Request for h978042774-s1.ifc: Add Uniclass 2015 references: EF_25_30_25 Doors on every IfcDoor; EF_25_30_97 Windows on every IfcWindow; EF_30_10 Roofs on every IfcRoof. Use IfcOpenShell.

First a look at what the model holds.

```python
import ifcopenshell

model = ifcopenshell.open("h978042774-s1.ifc")
print(model.schema)
print("classifications:", [c.Name for c in model.by_type("IfcClassification")])
for ifc_class in ("IfcDoor", "IfcRoof", "IfcStair", "IfcWall", "IfcWindow"):
    print(ifc_class, len(model.by_type(ifc_class)))
```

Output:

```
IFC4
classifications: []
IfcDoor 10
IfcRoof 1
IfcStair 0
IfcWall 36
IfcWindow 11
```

```python
import ifcopenshell
import ifcopenshell.api.classification

model = ifcopenshell.open("h978042774-s1.ifc")

system = ifcopenshell.api.classification.add_classification(model, classification="Uniclass 2015")

codes = {
    "IfcDoor": ("EF_25_30_25", "Doors"),
    "IfcWindow": ("EF_25_30_97", "Windows"),
    "IfcRoof": ("EF_30_10", "Roofs"),
}
for ifc_class, (code, name) in codes.items():
    products = model.by_type(ifc_class)
    ifcopenshell.api.classification.add_reference(
        model, products=products, classification=system, identification=code, name=name
    )
    print(code, len(products))

model.write("h978042774-s1-out.ifc")
```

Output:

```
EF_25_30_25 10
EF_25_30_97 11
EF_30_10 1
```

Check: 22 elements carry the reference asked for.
